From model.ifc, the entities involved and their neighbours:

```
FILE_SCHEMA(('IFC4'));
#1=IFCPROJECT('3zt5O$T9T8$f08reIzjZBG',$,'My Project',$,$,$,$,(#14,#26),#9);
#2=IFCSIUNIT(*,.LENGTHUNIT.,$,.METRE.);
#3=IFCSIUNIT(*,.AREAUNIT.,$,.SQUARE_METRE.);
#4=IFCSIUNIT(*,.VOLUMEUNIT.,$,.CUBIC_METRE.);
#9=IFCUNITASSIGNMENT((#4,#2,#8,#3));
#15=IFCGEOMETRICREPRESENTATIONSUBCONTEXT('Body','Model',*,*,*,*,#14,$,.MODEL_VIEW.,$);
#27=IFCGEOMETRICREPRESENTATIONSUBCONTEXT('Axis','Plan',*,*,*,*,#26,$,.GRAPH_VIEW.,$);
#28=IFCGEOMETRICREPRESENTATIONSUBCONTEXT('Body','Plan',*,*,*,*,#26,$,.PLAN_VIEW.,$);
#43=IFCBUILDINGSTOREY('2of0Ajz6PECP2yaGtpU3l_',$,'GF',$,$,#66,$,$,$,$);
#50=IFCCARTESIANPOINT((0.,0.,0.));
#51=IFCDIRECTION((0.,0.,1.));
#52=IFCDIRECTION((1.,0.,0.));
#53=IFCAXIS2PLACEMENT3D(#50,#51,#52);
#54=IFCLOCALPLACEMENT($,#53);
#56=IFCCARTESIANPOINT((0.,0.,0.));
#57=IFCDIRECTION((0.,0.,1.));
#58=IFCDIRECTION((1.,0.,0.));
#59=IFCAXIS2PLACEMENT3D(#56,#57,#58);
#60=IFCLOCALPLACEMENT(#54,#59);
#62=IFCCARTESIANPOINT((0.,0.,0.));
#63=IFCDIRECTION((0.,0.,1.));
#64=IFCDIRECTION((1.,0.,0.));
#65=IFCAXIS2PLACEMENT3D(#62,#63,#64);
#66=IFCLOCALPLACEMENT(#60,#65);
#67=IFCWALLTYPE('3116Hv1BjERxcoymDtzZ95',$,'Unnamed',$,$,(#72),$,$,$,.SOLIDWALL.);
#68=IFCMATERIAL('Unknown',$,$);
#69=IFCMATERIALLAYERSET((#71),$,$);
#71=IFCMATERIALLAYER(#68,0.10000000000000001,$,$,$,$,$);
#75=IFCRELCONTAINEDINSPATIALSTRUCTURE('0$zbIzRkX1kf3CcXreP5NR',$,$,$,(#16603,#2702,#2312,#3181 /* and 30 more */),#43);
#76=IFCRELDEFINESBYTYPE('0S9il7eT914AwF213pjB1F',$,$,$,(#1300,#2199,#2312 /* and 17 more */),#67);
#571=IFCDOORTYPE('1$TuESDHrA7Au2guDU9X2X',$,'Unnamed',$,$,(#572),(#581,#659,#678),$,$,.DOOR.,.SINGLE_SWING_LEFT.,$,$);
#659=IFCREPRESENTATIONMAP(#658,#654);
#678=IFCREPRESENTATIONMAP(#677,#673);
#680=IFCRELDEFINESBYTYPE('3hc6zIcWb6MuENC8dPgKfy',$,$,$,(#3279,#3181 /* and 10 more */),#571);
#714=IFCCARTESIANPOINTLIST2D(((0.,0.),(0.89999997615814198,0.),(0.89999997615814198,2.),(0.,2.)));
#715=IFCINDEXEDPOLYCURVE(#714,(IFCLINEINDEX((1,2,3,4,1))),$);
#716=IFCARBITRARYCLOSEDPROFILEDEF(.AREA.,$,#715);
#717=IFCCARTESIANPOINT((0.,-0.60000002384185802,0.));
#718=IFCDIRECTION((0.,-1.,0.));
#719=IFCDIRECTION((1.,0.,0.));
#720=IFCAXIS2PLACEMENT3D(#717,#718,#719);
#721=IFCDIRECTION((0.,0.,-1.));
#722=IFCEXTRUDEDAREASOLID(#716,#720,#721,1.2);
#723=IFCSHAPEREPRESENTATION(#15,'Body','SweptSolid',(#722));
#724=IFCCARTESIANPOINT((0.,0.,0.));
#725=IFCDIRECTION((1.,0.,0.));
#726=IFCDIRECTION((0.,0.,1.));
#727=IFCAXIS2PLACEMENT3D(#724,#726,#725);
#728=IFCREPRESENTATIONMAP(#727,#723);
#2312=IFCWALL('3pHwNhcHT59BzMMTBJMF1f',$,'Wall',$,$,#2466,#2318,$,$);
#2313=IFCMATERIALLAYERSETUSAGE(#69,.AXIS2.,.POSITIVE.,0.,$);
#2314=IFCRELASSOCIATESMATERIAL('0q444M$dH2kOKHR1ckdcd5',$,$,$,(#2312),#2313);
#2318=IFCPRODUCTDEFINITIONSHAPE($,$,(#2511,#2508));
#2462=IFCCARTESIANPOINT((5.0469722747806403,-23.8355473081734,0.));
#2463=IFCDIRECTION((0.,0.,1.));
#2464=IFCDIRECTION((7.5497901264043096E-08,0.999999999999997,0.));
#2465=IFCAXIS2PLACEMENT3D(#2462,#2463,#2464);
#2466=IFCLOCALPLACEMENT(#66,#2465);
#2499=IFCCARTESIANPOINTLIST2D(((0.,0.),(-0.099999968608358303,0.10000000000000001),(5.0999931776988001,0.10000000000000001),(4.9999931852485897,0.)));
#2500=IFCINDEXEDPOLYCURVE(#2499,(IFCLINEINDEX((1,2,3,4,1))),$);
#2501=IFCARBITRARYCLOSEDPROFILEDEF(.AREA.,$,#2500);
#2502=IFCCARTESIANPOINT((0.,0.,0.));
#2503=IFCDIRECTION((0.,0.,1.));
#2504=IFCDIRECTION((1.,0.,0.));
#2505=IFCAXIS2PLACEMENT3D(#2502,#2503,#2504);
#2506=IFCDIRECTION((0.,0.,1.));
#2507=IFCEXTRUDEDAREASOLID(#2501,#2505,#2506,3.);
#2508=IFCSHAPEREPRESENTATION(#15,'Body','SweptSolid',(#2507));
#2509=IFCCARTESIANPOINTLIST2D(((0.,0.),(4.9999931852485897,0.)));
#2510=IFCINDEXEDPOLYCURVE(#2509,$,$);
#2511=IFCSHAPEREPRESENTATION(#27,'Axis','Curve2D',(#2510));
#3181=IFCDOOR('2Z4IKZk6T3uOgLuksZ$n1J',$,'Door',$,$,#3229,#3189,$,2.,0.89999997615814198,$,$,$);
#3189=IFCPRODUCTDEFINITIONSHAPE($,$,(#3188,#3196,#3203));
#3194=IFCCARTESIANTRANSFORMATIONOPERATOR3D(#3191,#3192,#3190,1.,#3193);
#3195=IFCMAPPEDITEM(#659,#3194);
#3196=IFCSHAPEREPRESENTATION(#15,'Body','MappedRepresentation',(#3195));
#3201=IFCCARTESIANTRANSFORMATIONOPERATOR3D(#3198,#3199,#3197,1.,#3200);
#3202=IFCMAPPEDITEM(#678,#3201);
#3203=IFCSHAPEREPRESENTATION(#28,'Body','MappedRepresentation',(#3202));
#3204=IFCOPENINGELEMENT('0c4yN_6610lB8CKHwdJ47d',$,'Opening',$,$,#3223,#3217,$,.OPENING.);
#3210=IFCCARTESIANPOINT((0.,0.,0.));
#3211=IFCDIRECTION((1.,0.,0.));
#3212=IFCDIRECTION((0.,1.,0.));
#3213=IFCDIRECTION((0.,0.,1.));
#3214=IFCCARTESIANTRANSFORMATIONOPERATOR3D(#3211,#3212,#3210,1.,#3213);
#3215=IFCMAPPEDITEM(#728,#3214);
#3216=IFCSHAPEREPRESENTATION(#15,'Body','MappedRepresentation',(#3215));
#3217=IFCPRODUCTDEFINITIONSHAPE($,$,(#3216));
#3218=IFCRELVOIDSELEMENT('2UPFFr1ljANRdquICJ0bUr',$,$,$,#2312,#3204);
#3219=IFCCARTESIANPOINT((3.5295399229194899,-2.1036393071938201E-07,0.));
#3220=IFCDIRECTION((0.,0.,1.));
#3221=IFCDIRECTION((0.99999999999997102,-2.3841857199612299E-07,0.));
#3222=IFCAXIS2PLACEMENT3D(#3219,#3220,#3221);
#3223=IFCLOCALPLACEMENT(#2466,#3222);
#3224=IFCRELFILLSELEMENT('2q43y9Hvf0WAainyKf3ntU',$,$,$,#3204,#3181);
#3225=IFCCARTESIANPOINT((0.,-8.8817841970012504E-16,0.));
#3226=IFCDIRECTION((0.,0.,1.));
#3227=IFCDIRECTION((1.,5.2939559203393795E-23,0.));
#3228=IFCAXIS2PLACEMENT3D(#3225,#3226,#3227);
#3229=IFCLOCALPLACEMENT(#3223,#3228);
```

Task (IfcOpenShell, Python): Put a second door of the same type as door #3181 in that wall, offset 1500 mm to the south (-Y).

```python
import ifcopenshell
import ifcopenshell.api.feature
import ifcopenshell.api.geometry
import ifcopenshell.api.root
import ifcopenshell.geom
import ifcopenshell.util.element
import ifcopenshell.util.placement
import ifcopenshell.util.shape
import ifcopenshell.util.unit

model = ifcopenshell.open("model.ifc")
unit_scale = ifcopenshell.util.unit.calculate_unit_scale(model)
settings = ifcopenshell.geom.settings()


def volume(element):
    """Net volume in cubic metres, openings subtracted."""
    shape = ifcopenshell.geom.create_shape(settings, element)
    return ifcopenshell.util.shape.get_volume(shape.geometry)


door = model.by_guid("2Z4IKZk6T3uOgLuksZ$n1J")
opening = door.FillsVoids[0].RelatingOpeningElement
wall = opening.VoidsElements[0].RelatingBuildingElement
before = volume(wall)
shift = ifcopenshell.util.placement.get_local_placement(wall.ObjectPlacement)[:3, 0] * -1.5 / unit_scale

# copy_class copies the void relationship, type, container and properties, but no geometry.
new_opening = ifcopenshell.api.root.copy_class(model, product=opening)
new_opening.Representation = ifcopenshell.util.element.copy_deep(
    model, opening.Representation, exclude=["IfcGeometricRepresentationContext", "IfcRepresentationMap"]
)
new_door = ifcopenshell.api.root.copy_class(model, product=door)
new_door.Representation = ifcopenshell.util.element.copy_deep(
    model, door.Representation, exclude=["IfcGeometricRepresentationContext", "IfcRepresentationMap"]
)
ifcopenshell.api.feature.add_filling(model, opening=new_opening, element=new_door)

for old, new in ((opening, new_opening), (door, new_door)):
    matrix = ifcopenshell.util.placement.get_local_placement(old.ObjectPlacement)
    matrix[:3, 3] += shift
    ifcopenshell.api.geometry.edit_object_placement(model, product=new, matrix=matrix, is_si=False)

after = volume(wall)

print(f"wall volume {before:.3f} -> {after:.3f} m3")

model.write("model_updated.ifc")
```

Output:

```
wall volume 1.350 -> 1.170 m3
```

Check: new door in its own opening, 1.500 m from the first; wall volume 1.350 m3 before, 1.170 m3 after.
